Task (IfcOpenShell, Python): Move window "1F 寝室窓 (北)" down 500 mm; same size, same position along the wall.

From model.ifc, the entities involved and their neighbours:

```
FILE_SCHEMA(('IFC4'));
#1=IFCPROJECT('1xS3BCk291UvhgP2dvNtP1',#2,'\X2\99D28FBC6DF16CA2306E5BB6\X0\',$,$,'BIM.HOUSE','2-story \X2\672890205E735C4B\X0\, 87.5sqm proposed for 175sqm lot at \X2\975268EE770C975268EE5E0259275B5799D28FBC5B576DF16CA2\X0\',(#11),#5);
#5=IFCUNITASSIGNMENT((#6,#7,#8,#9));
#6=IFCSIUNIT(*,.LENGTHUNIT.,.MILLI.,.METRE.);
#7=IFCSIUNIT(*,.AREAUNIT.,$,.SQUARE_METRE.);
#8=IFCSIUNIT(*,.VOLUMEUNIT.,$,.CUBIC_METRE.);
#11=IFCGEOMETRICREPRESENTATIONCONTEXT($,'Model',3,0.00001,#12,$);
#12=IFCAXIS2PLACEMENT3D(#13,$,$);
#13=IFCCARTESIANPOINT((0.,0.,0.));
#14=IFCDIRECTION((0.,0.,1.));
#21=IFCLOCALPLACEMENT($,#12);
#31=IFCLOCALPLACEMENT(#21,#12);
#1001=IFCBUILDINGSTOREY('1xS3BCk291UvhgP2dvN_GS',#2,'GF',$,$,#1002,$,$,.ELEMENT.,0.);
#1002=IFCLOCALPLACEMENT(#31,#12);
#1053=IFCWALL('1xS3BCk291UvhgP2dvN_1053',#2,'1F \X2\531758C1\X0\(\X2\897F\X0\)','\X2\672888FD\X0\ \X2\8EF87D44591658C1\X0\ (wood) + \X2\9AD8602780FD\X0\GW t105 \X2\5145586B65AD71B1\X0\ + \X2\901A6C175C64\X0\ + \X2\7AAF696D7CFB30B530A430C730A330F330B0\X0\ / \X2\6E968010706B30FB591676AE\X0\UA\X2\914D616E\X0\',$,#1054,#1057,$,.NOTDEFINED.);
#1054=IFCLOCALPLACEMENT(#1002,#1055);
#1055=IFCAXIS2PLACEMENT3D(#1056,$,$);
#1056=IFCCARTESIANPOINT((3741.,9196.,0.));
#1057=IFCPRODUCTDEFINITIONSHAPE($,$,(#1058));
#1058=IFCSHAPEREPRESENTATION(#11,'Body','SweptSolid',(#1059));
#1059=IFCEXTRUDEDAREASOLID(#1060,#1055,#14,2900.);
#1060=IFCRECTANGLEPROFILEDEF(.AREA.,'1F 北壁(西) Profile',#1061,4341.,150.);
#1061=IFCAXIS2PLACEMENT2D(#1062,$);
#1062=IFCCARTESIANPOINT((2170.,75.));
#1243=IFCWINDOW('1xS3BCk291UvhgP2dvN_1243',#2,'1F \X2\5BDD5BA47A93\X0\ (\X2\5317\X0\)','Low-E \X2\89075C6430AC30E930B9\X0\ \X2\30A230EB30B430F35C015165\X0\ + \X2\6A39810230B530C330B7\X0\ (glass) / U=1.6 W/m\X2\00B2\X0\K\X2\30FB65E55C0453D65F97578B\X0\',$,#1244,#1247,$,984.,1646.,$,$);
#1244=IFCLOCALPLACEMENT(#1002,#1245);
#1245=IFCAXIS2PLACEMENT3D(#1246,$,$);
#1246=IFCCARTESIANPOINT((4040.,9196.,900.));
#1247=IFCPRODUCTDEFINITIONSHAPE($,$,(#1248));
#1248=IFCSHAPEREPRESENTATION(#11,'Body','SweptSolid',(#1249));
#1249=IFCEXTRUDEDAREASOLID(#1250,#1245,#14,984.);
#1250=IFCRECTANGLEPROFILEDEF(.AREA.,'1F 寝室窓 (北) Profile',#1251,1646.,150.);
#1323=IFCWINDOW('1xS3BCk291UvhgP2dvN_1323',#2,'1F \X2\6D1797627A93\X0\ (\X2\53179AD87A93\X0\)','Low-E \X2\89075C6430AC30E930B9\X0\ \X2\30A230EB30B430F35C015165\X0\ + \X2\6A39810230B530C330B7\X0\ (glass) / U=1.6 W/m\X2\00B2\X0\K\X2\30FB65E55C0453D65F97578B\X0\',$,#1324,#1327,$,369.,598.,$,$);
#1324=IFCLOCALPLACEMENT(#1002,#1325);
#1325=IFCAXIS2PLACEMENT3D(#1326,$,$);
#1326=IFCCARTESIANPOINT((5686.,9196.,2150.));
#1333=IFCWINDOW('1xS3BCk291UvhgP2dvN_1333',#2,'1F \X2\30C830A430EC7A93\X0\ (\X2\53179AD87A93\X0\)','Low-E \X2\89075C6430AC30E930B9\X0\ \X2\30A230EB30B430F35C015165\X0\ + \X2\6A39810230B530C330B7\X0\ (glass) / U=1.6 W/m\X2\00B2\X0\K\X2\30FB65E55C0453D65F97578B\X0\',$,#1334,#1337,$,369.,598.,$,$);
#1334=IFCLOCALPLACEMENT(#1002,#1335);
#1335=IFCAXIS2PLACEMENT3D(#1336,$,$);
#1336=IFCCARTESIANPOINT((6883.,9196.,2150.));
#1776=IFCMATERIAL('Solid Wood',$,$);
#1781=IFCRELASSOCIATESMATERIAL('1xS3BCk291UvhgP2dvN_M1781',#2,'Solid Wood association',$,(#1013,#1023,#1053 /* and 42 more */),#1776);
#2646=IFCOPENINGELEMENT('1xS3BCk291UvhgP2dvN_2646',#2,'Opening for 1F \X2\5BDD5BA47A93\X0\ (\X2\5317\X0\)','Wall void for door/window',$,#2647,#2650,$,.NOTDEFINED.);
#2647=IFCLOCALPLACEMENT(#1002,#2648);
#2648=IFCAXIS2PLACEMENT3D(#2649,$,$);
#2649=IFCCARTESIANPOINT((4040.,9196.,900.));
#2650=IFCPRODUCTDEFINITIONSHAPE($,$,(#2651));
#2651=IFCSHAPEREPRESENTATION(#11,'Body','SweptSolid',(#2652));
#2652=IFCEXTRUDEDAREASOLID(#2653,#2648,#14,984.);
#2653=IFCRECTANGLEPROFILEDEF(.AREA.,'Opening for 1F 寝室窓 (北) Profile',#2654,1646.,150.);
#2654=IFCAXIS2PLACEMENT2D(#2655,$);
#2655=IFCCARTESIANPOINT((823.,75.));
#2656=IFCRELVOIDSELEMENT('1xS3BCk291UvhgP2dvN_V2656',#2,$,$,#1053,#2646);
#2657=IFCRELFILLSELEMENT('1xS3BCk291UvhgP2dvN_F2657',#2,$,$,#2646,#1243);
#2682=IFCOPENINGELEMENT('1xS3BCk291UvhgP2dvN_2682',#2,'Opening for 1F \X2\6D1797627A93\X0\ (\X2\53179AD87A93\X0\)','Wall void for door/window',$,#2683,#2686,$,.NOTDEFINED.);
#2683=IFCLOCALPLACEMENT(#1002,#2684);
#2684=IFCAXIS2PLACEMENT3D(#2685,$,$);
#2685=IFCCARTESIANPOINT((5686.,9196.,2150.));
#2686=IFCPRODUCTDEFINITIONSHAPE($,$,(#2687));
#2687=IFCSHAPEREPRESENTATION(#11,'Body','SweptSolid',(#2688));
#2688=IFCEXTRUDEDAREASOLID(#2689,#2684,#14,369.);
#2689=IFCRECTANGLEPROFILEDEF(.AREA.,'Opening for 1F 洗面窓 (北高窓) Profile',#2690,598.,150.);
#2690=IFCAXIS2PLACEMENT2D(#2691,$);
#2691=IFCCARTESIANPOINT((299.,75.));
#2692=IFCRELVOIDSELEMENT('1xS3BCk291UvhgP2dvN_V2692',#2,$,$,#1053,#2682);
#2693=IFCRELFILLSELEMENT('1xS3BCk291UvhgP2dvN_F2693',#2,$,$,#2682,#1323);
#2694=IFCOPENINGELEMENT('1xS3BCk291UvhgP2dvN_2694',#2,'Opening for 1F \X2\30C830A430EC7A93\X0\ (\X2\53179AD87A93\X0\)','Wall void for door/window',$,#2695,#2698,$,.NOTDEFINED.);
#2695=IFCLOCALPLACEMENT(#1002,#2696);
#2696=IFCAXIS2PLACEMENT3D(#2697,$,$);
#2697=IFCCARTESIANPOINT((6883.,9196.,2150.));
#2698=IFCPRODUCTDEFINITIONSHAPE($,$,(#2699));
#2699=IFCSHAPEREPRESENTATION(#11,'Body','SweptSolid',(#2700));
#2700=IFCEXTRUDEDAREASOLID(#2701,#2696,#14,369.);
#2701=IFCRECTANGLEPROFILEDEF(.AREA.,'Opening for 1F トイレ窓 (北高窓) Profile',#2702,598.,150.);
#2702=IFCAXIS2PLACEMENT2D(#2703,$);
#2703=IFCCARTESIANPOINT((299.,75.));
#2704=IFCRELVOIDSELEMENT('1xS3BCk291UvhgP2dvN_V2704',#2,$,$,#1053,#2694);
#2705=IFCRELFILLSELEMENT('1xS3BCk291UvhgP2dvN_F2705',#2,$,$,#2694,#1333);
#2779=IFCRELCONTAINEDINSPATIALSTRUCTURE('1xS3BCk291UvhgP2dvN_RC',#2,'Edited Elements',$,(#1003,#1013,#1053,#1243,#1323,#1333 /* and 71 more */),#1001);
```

```python
import numpy as np
import ifcopenshell
import ifcopenshell.api.geometry
import ifcopenshell.util.placement
import ifcopenshell.util.unit

model = ifcopenshell.open("model.ifc")
unit_scale = ifcopenshell.util.unit.calculate_unit_scale(model)

window = model.by_guid("1xS3BCk291UvhgP2dvN_1243")
opening = window.FillsVoids[0].RelatingOpeningElement
dz = -500.0

shift = np.array([0.0, 0.0, dz])
# The window is not placed relative to its opening, so move both.
for product in (opening, window):
    matrix = ifcopenshell.util.placement.get_local_placement(product.ObjectPlacement)
    matrix[:3, 3] += shift
    ifcopenshell.api.geometry.edit_object_placement(model, product=product, matrix=matrix, is_si=False)

print(f"moved by {dz * unit_scale:+.3f} m")

model.write("model_v2.ifc")
```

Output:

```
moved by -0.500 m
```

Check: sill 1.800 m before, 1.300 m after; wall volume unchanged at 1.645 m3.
